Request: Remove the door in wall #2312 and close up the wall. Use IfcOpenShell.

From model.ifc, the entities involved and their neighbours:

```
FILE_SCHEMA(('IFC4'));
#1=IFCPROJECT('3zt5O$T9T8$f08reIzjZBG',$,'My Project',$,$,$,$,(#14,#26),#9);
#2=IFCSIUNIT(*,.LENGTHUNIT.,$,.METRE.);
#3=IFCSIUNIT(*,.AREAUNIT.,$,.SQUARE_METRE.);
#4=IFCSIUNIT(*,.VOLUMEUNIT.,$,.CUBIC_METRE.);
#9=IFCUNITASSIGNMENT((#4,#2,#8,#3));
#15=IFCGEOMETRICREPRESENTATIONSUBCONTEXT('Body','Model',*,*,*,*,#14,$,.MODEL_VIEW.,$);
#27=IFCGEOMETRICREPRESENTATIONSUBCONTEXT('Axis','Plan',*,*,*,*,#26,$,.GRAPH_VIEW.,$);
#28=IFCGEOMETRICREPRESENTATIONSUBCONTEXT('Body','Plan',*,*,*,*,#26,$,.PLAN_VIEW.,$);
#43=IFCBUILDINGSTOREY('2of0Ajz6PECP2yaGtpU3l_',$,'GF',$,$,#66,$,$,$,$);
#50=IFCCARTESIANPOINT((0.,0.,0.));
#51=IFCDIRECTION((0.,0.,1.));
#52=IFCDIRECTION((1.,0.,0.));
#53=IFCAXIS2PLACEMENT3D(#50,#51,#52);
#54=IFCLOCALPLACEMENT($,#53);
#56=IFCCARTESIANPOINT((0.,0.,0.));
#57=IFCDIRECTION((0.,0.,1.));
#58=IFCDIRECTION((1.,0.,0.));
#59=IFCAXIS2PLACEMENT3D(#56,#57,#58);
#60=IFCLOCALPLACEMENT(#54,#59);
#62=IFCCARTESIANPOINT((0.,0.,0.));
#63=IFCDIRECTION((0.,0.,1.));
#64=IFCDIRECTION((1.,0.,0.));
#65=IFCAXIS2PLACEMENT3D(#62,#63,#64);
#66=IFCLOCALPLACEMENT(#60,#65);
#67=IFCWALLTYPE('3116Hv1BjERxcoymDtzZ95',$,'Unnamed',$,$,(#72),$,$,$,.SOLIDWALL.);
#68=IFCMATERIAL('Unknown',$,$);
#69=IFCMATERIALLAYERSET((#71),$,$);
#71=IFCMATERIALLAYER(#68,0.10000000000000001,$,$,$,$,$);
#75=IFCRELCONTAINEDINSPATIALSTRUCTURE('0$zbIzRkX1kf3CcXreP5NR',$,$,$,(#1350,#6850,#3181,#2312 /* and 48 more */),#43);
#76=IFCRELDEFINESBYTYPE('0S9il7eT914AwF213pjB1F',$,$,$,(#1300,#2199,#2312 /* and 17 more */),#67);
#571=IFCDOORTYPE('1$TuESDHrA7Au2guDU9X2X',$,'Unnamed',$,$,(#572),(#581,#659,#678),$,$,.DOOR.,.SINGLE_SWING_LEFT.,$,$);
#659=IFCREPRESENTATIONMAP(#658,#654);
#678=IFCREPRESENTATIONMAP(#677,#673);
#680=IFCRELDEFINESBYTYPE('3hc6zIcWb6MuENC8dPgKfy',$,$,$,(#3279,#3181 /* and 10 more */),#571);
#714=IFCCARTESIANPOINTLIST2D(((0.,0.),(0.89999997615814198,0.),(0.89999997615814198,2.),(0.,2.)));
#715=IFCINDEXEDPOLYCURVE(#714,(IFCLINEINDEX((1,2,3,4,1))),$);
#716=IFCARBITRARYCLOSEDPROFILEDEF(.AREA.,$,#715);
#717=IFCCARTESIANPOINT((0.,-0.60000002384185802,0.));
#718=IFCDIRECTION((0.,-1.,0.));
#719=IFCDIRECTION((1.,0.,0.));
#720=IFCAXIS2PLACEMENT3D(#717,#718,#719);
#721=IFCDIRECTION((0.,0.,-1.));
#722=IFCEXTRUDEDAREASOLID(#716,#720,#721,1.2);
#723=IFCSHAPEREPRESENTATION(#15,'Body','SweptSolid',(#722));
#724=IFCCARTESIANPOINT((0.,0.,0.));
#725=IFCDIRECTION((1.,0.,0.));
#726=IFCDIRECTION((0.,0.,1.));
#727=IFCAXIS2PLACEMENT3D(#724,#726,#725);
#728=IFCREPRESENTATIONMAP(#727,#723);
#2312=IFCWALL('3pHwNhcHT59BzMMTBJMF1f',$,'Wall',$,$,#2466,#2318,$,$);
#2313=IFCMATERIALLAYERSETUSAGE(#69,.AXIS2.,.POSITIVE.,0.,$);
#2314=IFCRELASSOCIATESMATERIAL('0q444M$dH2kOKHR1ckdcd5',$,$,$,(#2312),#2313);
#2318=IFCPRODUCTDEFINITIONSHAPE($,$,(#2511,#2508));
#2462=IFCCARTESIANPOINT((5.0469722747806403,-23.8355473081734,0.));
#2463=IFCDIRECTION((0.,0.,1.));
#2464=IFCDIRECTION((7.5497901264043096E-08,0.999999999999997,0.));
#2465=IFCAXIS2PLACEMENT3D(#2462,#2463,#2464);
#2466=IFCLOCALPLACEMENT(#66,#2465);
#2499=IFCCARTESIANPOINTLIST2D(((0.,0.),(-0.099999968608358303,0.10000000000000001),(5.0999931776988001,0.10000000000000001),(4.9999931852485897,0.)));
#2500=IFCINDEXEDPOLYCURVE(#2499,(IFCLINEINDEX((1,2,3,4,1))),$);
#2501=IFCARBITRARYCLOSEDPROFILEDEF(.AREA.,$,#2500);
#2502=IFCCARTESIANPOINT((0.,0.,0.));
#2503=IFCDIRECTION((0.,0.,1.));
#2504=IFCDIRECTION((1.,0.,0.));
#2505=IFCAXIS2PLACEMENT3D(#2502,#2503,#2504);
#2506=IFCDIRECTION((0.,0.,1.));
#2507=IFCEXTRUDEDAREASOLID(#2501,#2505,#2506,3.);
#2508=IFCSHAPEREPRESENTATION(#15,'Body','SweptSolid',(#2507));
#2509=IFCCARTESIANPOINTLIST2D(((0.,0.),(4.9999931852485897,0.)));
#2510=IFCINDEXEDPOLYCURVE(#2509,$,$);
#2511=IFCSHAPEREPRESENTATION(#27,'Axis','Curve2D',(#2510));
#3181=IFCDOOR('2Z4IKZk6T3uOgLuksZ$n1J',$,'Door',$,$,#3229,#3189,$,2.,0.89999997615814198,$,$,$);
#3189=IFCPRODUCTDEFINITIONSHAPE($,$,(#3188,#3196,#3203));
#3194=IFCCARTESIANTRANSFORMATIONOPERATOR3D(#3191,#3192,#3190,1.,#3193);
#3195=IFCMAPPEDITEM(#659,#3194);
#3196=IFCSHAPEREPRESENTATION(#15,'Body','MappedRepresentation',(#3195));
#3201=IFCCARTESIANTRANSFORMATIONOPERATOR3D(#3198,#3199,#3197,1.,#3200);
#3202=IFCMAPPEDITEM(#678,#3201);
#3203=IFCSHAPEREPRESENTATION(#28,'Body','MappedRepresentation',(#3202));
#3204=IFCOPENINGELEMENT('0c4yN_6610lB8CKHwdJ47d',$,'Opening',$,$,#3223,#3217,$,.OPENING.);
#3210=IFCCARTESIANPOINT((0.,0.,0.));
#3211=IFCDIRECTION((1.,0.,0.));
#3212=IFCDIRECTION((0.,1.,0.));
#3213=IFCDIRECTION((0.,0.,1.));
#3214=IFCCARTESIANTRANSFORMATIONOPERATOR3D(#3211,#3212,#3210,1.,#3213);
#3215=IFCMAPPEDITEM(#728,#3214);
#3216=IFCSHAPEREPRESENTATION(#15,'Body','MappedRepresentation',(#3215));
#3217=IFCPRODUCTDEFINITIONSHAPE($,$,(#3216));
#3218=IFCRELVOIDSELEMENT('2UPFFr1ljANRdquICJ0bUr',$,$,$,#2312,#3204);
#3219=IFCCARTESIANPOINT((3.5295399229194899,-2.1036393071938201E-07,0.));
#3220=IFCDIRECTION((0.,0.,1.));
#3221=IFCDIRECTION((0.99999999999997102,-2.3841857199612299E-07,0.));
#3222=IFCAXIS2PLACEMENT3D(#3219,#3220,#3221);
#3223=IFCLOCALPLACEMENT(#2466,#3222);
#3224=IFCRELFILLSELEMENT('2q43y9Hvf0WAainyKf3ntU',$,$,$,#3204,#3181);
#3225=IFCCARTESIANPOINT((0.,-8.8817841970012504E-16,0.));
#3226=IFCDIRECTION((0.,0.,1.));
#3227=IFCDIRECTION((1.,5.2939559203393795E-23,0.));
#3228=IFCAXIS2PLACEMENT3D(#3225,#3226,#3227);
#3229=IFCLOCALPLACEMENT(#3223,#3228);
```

```python
import ifcopenshell
import ifcopenshell.api.feature
import ifcopenshell.api.root
import ifcopenshell.geom
import ifcopenshell.util.shape

model = ifcopenshell.open("model.ifc")
settings = ifcopenshell.geom.settings()


def volume(element):
    """Net volume in cubic metres, openings subtracted."""
    shape = ifcopenshell.geom.create_shape(settings, element)
    return ifcopenshell.util.shape.get_volume(shape.geometry)


door = model.by_id(3181)
opening = door.FillsVoids[0].RelatingOpeningElement
wall = opening.VoidsElements[0].RelatingBuildingElement
before = volume(wall)

ifcopenshell.api.root.remove_product(model, product=door)
ifcopenshell.api.feature.remove_feature(model, feature=opening)

after = volume(wall)

print(f"wall volume {before:.3f} -> {after:.3f} m3")

model.write("model_edited.ifc")
```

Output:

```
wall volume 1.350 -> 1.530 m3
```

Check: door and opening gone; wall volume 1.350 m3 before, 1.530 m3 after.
